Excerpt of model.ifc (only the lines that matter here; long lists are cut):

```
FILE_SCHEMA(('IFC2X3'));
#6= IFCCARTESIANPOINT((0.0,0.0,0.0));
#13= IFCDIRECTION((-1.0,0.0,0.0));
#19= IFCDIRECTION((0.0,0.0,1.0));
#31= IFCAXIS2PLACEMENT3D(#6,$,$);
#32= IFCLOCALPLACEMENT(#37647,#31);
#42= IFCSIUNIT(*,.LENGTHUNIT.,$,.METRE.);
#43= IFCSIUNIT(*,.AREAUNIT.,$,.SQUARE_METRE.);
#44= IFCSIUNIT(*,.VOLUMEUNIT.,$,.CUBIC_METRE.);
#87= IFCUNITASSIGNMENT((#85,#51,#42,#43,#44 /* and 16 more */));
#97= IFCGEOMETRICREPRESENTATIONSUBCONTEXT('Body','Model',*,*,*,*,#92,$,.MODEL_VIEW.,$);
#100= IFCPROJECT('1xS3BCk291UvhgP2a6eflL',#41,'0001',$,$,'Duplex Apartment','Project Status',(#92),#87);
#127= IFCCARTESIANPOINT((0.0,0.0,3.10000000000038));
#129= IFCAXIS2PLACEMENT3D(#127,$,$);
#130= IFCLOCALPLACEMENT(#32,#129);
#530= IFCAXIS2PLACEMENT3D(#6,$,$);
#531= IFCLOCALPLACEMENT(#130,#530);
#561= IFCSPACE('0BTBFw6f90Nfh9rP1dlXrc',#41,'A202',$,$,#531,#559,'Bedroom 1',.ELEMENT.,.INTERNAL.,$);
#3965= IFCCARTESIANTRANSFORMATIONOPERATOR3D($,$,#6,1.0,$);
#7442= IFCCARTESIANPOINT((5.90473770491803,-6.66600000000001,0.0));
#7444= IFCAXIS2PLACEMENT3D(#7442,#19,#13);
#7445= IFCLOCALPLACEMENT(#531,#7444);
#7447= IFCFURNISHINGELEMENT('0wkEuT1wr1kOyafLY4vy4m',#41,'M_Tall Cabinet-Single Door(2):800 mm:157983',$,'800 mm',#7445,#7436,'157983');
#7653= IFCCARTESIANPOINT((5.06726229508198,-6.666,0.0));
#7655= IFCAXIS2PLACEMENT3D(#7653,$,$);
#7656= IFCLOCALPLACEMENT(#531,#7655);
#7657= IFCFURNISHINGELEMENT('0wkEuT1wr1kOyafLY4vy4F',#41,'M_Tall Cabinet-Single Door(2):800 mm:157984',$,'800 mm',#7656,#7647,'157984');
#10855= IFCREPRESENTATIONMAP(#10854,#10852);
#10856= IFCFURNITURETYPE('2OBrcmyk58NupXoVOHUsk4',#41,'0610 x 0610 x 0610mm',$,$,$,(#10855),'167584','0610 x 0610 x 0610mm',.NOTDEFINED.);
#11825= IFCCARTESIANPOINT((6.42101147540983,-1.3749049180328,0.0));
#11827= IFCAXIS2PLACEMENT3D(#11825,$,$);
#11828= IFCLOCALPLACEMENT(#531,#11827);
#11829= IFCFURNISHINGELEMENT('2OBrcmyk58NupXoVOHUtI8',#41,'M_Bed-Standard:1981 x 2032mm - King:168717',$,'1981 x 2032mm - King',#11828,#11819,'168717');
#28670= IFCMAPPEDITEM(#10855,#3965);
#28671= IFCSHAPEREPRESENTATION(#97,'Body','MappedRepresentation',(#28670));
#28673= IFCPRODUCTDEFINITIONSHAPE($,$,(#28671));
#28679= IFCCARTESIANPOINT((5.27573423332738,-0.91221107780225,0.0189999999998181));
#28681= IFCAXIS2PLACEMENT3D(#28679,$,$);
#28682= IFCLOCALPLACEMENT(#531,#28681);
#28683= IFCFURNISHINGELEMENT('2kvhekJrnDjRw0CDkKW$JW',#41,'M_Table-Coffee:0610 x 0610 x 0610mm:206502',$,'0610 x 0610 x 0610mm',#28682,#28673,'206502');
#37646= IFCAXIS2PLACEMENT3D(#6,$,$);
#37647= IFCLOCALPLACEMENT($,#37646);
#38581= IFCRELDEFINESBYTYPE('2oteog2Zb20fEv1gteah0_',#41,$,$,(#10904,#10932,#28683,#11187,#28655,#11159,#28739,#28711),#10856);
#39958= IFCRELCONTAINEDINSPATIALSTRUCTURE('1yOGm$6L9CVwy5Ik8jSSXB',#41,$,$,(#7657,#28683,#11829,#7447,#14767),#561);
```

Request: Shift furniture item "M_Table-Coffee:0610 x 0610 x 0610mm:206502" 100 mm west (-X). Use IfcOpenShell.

```python
import ifcopenshell
import ifcopenshell.api.geometry
import ifcopenshell.util.placement

model = ifcopenshell.open("model.ifc")

item = model.by_guid("2kvhekJrnDjRw0CDkKW$JW")
matrix = ifcopenshell.util.placement.get_local_placement(item.ObjectPlacement)
matrix[0, 3] -= 0.1
ifcopenshell.api.geometry.edit_object_placement(model, product=item, matrix=matrix, is_si=False)

print(ifcopenshell.util.placement.get_local_placement(item.ObjectPlacement).round(3) + 0.0)

model.write("model_v2.ifc")
```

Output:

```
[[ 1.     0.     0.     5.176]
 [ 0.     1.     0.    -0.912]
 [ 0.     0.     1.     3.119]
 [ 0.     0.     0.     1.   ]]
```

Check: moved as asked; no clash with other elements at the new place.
